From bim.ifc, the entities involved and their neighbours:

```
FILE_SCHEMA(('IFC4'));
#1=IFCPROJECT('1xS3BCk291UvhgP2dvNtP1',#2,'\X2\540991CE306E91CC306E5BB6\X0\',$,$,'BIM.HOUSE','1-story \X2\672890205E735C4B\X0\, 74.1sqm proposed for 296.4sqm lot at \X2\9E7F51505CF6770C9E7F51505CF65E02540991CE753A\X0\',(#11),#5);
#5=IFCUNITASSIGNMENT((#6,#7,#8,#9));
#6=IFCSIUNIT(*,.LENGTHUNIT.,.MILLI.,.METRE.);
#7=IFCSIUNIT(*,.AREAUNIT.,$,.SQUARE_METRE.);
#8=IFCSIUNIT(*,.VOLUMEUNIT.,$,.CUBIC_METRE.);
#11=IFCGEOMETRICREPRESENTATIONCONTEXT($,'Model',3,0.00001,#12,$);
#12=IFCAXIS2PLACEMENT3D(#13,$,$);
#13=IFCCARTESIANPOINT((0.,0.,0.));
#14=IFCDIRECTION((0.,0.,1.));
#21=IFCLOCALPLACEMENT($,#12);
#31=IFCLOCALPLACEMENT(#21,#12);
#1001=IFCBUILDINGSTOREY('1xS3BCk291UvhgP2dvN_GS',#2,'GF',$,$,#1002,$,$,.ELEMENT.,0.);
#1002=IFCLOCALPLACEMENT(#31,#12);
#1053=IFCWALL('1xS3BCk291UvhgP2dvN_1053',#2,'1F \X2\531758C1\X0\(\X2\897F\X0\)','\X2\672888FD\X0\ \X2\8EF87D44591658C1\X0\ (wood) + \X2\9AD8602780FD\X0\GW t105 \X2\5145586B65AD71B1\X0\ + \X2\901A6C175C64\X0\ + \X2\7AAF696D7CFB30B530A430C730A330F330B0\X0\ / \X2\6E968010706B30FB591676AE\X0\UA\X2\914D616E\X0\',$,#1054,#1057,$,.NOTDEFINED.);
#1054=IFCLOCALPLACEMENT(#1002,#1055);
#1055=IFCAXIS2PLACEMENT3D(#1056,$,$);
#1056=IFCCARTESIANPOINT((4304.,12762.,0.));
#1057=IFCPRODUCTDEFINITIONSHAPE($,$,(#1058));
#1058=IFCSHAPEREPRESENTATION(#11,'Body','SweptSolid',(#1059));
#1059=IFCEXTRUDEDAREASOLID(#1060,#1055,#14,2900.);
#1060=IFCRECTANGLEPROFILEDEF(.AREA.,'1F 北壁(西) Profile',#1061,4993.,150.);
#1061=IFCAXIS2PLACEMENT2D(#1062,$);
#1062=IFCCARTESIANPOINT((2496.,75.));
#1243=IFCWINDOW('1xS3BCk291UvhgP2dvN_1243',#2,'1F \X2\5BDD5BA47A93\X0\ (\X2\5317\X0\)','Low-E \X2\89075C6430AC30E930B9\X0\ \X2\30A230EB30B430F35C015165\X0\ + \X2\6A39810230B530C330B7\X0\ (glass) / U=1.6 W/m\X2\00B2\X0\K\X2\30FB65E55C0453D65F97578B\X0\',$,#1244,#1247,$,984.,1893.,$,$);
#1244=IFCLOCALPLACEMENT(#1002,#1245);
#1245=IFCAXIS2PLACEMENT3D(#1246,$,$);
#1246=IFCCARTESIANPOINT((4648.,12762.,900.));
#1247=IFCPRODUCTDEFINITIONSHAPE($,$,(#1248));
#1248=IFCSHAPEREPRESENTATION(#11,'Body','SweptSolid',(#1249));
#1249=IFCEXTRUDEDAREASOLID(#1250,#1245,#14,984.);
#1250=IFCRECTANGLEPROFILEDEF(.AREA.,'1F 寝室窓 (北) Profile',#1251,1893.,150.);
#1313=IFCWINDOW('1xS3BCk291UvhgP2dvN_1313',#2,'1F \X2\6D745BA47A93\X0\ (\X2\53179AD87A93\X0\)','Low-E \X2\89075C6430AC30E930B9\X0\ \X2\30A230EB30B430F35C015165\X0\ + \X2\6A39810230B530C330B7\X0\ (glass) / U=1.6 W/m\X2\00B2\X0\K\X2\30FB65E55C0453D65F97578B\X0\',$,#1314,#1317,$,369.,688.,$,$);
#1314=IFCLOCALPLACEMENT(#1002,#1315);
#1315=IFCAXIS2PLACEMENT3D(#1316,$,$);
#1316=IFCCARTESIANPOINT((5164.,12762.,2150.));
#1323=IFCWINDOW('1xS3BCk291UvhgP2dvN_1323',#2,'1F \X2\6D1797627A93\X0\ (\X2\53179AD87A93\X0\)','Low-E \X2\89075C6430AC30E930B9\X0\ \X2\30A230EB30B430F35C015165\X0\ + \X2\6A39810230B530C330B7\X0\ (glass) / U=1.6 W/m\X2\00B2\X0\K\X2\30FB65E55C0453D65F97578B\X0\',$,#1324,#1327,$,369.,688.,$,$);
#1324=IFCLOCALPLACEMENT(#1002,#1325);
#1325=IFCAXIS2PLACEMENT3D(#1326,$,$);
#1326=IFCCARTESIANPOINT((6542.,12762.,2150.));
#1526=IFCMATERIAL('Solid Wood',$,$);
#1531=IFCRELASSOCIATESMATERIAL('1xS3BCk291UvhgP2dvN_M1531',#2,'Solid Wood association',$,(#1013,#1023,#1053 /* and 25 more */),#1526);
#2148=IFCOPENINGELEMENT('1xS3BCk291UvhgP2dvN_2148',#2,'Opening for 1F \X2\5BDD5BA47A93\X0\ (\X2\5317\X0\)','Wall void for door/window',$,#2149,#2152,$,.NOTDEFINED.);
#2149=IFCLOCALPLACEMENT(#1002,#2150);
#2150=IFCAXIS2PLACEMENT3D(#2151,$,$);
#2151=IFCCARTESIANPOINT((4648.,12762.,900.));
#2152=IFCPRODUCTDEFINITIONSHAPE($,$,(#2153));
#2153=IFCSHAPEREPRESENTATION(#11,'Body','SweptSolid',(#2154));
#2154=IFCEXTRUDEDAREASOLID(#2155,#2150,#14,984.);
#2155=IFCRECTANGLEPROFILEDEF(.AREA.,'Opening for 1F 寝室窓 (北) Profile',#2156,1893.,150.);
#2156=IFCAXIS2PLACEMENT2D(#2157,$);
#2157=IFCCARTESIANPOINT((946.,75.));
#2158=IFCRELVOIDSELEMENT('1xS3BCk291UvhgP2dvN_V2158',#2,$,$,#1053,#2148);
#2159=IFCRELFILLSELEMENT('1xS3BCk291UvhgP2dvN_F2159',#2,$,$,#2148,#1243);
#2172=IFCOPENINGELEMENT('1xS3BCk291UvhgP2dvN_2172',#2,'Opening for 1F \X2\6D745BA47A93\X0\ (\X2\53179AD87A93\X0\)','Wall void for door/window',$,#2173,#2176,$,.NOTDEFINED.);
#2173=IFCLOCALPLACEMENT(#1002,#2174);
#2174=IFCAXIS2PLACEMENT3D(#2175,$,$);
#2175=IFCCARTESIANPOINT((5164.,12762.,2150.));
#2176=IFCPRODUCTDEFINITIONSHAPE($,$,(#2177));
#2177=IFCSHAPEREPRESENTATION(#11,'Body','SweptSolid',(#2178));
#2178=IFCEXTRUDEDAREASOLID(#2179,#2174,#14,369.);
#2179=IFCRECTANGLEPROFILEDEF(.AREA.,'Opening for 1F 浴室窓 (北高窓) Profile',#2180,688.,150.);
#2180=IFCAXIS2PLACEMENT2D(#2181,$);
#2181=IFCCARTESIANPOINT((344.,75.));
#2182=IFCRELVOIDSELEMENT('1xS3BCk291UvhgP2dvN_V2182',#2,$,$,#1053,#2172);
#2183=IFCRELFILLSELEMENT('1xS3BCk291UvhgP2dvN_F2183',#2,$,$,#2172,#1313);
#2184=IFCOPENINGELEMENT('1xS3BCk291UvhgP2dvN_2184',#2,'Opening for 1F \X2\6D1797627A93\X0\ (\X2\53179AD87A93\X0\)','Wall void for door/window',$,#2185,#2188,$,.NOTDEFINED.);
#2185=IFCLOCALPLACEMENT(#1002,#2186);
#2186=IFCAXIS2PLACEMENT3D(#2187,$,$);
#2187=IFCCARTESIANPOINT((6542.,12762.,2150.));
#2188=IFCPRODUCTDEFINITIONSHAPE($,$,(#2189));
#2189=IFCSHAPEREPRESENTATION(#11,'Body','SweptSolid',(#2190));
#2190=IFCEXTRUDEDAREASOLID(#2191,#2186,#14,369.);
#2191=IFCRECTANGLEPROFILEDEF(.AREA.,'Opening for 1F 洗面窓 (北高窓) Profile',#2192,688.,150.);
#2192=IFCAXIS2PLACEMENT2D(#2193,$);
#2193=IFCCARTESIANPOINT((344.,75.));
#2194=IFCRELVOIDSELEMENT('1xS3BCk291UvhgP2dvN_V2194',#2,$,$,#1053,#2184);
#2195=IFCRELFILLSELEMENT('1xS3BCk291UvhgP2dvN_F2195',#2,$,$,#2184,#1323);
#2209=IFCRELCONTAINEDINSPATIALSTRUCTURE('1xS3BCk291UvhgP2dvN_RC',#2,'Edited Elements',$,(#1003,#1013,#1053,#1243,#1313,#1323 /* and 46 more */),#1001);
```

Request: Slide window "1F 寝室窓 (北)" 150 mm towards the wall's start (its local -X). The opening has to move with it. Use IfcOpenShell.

```python
import ifcopenshell
import ifcopenshell.api.geometry
import ifcopenshell.util.placement
import ifcopenshell.util.unit

model = ifcopenshell.open("bim.ifc")
unit_scale = ifcopenshell.util.unit.calculate_unit_scale(model)

window = model.by_id(1243)
opening = window.FillsVoids[0].RelatingOpeningElement
wall = opening.VoidsElements[0].RelatingBuildingElement

wall_matrix = ifcopenshell.util.placement.get_local_placement(wall.ObjectPlacement)
shift = wall_matrix[:3, 0] * -0.15 / unit_scale
before = ifcopenshell.util.placement.get_local_placement(window.ObjectPlacement)[:3, 3].copy()

# The window is not placed relative to its opening, so move both.
for product in (opening, window):
    matrix = ifcopenshell.util.placement.get_local_placement(product.ObjectPlacement)
    matrix[:3, 3] += shift
    ifcopenshell.api.geometry.edit_object_placement(model, product=product, matrix=matrix, is_si=False)

after = ifcopenshell.util.placement.get_local_placement(window.ObjectPlacement)[:3, 3]
print("window moved by", (after - before).round(3) + 0.0)

model.write("bim_edited.ifc")
```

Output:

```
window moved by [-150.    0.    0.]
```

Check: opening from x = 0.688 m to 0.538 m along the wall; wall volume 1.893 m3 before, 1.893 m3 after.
